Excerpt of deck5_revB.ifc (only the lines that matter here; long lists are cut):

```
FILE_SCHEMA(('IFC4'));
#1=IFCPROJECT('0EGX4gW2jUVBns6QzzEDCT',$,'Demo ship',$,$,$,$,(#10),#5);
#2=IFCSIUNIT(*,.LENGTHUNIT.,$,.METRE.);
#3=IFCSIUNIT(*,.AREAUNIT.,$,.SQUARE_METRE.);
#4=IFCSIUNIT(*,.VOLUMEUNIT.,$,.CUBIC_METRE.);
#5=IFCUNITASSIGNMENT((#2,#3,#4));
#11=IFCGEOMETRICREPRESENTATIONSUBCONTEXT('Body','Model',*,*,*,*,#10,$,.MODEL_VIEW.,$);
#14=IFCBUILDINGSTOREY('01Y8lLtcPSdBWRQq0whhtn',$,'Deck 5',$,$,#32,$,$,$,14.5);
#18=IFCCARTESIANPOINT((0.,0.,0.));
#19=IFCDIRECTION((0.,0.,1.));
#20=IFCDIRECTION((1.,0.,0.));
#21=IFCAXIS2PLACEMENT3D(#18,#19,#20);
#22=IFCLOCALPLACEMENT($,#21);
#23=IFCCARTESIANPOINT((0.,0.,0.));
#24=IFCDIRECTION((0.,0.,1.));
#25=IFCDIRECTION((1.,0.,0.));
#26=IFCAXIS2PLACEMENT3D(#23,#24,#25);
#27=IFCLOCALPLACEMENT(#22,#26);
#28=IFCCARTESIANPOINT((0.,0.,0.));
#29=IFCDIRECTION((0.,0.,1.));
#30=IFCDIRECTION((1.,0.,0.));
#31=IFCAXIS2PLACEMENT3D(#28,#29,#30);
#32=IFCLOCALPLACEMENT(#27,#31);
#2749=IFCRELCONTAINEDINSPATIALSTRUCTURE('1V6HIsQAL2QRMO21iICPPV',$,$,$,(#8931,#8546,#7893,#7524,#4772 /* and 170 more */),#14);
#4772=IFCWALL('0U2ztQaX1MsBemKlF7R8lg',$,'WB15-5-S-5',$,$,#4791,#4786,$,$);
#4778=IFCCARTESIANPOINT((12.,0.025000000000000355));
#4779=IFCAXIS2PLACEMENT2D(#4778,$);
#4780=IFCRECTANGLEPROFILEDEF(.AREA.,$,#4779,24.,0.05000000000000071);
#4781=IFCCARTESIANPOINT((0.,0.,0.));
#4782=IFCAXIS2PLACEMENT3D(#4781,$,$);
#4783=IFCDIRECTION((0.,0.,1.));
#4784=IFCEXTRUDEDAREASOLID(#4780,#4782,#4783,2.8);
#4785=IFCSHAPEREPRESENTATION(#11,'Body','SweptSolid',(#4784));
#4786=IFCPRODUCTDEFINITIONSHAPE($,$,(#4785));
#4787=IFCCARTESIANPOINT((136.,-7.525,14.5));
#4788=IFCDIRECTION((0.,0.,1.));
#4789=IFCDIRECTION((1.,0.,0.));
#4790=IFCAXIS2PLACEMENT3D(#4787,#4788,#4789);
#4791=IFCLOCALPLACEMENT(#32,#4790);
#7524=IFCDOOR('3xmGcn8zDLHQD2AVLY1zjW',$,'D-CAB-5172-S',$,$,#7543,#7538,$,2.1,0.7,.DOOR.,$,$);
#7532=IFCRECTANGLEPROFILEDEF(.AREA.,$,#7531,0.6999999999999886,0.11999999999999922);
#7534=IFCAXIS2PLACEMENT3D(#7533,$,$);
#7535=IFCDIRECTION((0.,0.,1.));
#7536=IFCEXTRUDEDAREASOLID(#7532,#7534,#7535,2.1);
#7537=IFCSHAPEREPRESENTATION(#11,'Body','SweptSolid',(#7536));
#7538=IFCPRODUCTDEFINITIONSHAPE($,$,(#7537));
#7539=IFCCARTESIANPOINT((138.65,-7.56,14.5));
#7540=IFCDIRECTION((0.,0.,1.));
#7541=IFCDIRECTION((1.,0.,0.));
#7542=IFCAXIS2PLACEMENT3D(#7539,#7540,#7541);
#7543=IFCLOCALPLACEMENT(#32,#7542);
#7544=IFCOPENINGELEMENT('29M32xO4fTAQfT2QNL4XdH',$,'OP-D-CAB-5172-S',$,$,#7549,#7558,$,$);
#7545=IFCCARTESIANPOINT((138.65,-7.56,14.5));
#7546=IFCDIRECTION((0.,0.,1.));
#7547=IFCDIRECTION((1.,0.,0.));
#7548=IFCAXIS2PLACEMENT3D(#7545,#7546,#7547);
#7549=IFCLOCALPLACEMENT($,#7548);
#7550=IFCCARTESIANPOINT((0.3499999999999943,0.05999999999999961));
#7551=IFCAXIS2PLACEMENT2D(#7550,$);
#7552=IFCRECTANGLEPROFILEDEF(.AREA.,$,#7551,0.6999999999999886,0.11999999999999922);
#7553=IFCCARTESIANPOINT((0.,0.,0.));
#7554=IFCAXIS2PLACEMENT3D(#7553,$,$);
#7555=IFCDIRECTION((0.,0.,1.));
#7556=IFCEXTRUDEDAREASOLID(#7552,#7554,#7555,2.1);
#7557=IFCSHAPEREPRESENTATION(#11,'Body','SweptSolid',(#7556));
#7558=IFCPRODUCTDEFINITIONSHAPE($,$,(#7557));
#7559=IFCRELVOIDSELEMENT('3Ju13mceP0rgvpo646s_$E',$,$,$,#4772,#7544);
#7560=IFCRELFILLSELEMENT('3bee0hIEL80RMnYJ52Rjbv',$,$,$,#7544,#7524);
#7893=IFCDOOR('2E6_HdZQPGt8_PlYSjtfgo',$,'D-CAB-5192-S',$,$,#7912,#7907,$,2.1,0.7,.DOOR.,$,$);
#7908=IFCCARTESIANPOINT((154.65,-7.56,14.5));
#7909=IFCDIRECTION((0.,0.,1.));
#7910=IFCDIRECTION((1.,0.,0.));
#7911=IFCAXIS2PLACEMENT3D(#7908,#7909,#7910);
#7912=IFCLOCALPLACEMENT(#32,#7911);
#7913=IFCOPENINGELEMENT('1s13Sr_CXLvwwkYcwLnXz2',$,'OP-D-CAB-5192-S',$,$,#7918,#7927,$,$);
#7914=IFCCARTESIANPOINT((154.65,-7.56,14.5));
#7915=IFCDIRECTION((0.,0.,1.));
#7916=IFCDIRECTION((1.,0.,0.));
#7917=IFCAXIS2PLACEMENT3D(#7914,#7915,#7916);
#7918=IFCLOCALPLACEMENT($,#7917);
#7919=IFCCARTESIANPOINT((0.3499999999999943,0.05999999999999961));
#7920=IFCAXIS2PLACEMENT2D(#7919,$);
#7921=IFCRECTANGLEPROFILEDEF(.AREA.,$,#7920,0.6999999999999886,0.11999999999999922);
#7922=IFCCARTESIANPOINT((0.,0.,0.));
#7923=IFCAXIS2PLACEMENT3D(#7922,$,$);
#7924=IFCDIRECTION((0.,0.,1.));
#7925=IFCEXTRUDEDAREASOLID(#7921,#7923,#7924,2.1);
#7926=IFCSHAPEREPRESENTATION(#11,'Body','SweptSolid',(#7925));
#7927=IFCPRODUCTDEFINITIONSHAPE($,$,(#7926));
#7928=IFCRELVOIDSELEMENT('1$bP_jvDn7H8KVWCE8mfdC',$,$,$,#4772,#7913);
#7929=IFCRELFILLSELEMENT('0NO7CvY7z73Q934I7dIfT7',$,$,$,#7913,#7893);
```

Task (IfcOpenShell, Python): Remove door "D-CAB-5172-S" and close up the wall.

```python
import ifcopenshell
import ifcopenshell.api.feature
import ifcopenshell.api.root
import ifcopenshell.geom
import ifcopenshell.util.shape

model = ifcopenshell.open("deck5_revB.ifc")
settings = ifcopenshell.geom.settings()


def volume(element):
    """Net volume in cubic metres, openings subtracted."""
    shape = ifcopenshell.geom.create_shape(settings, element)
    return ifcopenshell.util.shape.get_volume(shape.geometry)


door = model.by_id(7524)
opening = door.FillsVoids[0].RelatingOpeningElement
wall = opening.VoidsElements[0].RelatingBuildingElement
before = volume(wall)

ifcopenshell.api.root.remove_product(model, product=door)
ifcopenshell.api.feature.remove_feature(model, feature=opening)

after = volume(wall)

print(f"wall volume {before:.3f} -> {after:.3f} m3")

model.write("deck5_revB_rev.ifc")
```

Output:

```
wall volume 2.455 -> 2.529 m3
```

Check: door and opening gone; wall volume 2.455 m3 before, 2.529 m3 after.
